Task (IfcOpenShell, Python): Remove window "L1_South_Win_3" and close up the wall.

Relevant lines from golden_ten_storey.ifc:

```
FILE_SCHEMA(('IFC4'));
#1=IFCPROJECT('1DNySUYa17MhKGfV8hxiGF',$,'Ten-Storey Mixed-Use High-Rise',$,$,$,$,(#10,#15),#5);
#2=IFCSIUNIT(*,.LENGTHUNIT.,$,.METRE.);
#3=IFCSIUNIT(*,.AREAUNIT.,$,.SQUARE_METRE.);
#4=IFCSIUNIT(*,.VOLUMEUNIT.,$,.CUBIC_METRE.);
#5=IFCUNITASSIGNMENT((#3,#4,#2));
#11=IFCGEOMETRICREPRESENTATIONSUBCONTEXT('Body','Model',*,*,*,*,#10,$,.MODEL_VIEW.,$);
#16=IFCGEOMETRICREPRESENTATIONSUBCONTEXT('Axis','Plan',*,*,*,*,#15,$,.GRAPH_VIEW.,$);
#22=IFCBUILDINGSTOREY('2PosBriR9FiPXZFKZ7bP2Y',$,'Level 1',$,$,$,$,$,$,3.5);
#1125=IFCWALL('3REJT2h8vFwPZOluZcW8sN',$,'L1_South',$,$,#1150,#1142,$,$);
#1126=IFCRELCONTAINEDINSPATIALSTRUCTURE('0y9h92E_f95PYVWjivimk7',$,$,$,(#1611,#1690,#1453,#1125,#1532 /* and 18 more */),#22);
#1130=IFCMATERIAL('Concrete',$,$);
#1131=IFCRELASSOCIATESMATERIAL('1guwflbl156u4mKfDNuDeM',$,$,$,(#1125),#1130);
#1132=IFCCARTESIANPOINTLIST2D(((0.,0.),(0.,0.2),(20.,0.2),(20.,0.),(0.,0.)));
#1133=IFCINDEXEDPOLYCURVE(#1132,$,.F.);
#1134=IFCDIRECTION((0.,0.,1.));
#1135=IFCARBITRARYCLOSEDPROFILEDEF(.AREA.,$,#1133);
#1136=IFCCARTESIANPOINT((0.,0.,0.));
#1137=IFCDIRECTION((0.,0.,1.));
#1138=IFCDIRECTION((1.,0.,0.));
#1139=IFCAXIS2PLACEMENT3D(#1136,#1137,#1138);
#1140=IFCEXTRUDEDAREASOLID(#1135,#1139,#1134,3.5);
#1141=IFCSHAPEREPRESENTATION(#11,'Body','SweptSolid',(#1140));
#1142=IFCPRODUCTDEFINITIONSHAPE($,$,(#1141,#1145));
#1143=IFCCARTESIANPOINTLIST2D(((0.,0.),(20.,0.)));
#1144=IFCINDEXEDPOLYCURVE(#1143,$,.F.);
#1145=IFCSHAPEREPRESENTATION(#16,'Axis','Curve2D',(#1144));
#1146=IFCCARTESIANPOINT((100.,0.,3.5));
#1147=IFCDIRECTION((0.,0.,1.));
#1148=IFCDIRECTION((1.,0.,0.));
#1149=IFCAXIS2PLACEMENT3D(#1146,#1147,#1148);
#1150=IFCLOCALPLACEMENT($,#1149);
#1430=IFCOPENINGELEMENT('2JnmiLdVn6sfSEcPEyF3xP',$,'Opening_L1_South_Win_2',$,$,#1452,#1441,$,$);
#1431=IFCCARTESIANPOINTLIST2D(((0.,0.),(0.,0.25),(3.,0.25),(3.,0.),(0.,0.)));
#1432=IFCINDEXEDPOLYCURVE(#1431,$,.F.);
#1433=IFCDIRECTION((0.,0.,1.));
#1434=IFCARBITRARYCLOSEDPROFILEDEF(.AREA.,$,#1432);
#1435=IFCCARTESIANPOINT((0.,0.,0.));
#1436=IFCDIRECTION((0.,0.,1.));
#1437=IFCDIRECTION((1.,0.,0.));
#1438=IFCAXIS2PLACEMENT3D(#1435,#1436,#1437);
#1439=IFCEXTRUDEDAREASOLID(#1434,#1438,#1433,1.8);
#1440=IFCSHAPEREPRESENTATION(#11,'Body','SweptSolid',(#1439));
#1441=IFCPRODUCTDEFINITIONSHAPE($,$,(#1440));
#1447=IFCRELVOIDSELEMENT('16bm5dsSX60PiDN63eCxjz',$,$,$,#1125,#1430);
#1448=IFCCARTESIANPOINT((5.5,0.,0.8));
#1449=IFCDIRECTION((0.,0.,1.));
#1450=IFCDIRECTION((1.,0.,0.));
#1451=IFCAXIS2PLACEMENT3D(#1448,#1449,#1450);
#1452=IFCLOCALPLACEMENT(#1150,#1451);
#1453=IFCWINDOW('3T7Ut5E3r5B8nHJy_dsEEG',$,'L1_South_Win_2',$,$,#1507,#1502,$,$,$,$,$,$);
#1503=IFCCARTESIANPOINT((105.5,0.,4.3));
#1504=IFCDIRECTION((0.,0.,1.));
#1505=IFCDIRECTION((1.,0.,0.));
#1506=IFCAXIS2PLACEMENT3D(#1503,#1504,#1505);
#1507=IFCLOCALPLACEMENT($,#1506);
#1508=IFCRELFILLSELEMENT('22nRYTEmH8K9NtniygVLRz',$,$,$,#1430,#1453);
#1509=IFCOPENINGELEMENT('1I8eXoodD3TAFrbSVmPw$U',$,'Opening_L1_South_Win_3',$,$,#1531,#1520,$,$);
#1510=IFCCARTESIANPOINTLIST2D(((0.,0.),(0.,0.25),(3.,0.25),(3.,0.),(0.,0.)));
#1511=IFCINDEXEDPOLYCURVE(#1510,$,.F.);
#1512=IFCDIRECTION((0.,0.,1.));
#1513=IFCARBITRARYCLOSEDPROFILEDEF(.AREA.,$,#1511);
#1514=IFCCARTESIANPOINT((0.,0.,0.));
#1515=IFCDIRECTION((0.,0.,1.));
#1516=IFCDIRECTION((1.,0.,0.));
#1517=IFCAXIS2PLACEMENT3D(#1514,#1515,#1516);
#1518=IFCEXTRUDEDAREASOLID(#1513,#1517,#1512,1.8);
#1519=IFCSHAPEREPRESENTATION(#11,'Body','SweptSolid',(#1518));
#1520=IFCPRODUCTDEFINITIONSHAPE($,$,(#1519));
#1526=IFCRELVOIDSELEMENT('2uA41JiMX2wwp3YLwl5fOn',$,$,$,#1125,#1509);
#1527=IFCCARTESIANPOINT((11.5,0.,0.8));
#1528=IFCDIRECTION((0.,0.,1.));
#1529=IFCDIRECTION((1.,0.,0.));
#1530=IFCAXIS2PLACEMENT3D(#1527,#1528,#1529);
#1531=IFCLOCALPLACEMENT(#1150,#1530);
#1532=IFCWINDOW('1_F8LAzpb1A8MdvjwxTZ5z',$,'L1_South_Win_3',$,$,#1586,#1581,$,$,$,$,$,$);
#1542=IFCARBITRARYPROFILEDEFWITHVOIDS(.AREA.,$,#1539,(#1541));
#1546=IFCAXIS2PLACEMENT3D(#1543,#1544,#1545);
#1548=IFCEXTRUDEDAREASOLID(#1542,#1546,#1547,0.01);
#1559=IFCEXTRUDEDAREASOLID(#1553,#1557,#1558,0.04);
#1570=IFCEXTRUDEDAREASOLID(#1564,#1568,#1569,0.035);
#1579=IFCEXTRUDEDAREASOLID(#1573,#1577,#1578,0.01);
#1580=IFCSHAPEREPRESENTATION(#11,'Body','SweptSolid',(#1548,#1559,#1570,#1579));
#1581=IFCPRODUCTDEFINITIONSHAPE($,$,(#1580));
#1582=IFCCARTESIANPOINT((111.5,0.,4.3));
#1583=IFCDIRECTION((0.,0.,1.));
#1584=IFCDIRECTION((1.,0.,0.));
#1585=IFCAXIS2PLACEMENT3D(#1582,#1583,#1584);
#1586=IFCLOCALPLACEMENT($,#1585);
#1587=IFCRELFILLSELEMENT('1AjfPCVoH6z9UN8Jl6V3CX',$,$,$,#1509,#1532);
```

```python
import ifcopenshell
import ifcopenshell.api.feature
import ifcopenshell.api.root
import ifcopenshell.geom
import ifcopenshell.util.shape

model = ifcopenshell.open("golden_ten_storey.ifc")
settings = ifcopenshell.geom.settings()


def volume(element):
    """Net volume in cubic metres, openings subtracted."""
    shape = ifcopenshell.geom.create_shape(settings, element)
    return ifcopenshell.util.shape.get_volume(shape.geometry)


window = model.by_guid("1_F8LAzpb1A8MdvjwxTZ5z")
opening = window.FillsVoids[0].RelatingOpeningElement
wall = opening.VoidsElements[0].RelatingBuildingElement
before = volume(wall)

ifcopenshell.api.root.remove_product(model, product=window)
ifcopenshell.api.feature.remove_feature(model, feature=opening)

after = volume(wall)

print(f"wall volume {before:.3f} -> {after:.3f} m3")

model.write("golden_ten_storey-out.ifc")
```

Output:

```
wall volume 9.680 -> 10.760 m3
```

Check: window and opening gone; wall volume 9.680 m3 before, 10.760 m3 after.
